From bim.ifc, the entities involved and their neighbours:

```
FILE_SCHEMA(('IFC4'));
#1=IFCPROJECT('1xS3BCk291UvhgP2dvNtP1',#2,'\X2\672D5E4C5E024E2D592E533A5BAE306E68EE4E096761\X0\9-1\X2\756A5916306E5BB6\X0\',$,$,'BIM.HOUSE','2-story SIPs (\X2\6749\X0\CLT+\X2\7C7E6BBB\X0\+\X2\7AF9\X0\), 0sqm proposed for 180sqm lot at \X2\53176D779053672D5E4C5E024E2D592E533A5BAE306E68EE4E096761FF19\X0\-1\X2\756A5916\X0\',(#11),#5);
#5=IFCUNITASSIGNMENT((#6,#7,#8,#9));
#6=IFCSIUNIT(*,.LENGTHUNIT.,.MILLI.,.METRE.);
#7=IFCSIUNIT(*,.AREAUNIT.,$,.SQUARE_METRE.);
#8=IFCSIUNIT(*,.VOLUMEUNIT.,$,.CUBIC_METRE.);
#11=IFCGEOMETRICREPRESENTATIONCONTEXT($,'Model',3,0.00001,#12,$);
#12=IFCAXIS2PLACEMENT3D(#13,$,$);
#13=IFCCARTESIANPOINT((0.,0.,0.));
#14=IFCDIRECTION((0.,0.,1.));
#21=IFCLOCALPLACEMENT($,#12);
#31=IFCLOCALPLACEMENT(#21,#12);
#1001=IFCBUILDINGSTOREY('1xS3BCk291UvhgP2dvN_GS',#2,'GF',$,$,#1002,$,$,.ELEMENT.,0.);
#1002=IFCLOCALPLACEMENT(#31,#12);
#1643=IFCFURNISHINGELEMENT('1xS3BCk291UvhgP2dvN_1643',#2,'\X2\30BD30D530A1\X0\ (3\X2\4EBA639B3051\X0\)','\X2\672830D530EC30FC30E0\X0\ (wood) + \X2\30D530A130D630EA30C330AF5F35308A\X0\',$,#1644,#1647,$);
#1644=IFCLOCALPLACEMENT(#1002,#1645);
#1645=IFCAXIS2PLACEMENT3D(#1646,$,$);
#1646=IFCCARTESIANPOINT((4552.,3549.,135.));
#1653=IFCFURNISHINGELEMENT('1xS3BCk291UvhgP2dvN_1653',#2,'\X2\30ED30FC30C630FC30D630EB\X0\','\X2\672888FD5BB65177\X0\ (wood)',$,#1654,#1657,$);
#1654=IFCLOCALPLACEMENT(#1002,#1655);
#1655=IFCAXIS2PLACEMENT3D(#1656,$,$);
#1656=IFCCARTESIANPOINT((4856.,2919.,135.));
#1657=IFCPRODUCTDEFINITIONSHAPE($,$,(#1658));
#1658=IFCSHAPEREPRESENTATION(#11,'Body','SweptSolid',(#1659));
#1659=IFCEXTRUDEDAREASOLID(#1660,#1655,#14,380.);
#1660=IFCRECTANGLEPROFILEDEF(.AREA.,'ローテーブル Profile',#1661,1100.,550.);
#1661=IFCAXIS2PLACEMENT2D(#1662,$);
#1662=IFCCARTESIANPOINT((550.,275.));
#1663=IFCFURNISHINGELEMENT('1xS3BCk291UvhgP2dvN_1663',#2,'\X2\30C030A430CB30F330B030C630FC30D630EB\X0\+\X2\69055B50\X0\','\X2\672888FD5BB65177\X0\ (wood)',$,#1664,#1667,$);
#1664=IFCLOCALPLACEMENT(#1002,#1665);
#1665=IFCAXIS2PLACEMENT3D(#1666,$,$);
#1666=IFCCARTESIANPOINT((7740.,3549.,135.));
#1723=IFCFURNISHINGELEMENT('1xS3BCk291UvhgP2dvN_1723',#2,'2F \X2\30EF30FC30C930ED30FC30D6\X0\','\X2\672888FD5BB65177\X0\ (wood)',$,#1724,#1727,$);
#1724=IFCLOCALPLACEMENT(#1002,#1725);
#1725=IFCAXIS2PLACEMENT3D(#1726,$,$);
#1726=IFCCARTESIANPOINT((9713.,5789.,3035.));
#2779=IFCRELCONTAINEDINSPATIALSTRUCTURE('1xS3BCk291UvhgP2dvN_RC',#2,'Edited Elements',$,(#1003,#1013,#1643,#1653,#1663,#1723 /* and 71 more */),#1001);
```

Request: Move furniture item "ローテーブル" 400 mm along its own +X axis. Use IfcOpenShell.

```python
import ifcopenshell
import ifcopenshell.api.geometry
import ifcopenshell.util.placement
import ifcopenshell.util.unit

model = ifcopenshell.open("bim.ifc")
unit_scale = ifcopenshell.util.unit.calculate_unit_scale(model)

item = model.by_id(1653)
matrix = ifcopenshell.util.placement.get_local_placement(item.ObjectPlacement)
matrix[:3, 3] += matrix[:3, 0] * 0.4 / unit_scale
ifcopenshell.api.geometry.edit_object_placement(model, product=item, matrix=matrix, is_si=False)

print(ifcopenshell.util.placement.get_local_placement(item.ObjectPlacement).round(3) + 0.0)

model.write("bim_updated.ifc")
```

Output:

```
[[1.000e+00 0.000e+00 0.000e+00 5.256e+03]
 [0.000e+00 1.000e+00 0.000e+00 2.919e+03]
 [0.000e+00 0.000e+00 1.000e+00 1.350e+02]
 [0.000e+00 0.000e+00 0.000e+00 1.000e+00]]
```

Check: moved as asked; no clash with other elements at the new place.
